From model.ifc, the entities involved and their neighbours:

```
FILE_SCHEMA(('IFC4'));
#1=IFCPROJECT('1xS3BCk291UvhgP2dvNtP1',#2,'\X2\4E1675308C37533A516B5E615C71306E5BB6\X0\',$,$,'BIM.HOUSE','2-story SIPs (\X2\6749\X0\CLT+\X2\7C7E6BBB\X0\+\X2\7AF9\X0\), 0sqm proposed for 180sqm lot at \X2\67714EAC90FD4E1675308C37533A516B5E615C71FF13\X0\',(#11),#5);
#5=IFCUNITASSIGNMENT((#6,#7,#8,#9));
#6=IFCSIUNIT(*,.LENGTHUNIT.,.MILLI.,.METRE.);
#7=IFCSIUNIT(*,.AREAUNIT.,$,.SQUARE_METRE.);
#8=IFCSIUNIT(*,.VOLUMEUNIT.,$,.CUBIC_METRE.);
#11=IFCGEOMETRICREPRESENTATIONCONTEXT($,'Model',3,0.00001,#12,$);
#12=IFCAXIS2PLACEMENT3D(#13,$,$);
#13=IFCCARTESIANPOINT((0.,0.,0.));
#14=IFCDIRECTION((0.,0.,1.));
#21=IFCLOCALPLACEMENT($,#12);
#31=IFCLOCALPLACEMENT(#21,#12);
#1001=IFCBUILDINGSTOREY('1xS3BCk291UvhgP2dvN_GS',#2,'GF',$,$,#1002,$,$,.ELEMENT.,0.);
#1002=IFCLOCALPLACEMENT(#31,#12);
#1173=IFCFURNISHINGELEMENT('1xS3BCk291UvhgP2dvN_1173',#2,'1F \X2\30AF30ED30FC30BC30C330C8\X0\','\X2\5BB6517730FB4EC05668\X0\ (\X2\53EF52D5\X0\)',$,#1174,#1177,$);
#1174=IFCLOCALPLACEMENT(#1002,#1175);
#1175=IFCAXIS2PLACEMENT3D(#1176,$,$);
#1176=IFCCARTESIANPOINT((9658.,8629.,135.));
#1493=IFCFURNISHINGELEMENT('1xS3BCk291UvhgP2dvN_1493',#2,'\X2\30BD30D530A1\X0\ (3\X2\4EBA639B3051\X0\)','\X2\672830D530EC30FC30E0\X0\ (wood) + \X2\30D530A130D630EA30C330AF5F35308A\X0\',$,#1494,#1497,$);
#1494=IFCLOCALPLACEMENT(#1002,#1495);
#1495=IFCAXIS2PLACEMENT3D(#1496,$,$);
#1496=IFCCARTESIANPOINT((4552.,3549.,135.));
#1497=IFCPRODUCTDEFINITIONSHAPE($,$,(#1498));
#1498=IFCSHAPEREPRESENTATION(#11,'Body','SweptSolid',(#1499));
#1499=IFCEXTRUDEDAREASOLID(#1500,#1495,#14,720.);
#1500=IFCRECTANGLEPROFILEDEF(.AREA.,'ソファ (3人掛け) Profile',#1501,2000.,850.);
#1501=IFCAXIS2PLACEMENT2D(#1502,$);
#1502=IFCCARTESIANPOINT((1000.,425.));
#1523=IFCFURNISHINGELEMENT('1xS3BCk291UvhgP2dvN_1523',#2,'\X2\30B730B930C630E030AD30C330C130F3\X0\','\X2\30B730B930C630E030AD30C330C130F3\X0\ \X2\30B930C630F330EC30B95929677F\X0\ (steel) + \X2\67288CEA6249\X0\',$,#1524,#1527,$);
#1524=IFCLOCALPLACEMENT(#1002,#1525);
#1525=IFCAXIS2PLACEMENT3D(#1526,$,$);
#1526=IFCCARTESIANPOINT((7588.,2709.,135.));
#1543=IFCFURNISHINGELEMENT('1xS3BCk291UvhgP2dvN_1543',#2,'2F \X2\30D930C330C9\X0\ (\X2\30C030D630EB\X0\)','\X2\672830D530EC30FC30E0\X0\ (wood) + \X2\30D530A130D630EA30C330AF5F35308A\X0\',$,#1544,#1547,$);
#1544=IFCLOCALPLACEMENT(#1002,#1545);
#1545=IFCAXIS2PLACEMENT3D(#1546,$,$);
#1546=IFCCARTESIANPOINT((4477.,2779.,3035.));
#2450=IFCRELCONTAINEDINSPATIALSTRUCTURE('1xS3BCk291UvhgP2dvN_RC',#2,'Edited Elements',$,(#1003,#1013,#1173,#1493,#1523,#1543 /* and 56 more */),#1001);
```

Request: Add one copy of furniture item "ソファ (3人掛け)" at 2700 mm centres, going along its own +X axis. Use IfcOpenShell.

```python
import ifcopenshell
import ifcopenshell.api.geometry
import ifcopenshell.api.root
import ifcopenshell.util.element
import ifcopenshell.util.placement
import ifcopenshell.util.unit

model = ifcopenshell.open("model.ifc")
unit_scale = ifcopenshell.util.unit.calculate_unit_scale(model)


def reuse_history(source, copy):
    """copy_class also copies each property set's owner history, people and application; keep the originals."""
    for rel in copy.IsDefinedBy:
        if rel.is_a("IfcRelDefinesByProperties") and (history := rel.RelatingPropertyDefinition.OwnerHistory):
            rel.RelatingPropertyDefinition.OwnerHistory = source.OwnerHistory
            ifcopenshell.util.element.remove_deep2(model, history)


source = model.by_guid("1xS3BCk291UvhgP2dvN_1493")
base = ifcopenshell.util.placement.get_local_placement(source.ObjectPlacement)
step = base[:3, 0] * 2.7 / unit_scale

for i in range(1, 2):
    copy = ifcopenshell.api.root.copy_class(model, product=source)
    copy.Representation = ifcopenshell.util.element.copy_deep(
        model, source.Representation, exclude=["IfcGeometricRepresentationContext", "IfcRepresentationMap"]
    )
    reuse_history(source, copy)
    matrix = base.copy()
    matrix[:3, 3] += i * step
    print("added at", matrix[:3, 3].round(3) + 0.0)
    ifcopenshell.api.geometry.edit_object_placement(model, product=copy, matrix=matrix, is_si=False)

model.write("model_v2.ifc")
```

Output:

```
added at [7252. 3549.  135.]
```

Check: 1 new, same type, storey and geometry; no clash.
